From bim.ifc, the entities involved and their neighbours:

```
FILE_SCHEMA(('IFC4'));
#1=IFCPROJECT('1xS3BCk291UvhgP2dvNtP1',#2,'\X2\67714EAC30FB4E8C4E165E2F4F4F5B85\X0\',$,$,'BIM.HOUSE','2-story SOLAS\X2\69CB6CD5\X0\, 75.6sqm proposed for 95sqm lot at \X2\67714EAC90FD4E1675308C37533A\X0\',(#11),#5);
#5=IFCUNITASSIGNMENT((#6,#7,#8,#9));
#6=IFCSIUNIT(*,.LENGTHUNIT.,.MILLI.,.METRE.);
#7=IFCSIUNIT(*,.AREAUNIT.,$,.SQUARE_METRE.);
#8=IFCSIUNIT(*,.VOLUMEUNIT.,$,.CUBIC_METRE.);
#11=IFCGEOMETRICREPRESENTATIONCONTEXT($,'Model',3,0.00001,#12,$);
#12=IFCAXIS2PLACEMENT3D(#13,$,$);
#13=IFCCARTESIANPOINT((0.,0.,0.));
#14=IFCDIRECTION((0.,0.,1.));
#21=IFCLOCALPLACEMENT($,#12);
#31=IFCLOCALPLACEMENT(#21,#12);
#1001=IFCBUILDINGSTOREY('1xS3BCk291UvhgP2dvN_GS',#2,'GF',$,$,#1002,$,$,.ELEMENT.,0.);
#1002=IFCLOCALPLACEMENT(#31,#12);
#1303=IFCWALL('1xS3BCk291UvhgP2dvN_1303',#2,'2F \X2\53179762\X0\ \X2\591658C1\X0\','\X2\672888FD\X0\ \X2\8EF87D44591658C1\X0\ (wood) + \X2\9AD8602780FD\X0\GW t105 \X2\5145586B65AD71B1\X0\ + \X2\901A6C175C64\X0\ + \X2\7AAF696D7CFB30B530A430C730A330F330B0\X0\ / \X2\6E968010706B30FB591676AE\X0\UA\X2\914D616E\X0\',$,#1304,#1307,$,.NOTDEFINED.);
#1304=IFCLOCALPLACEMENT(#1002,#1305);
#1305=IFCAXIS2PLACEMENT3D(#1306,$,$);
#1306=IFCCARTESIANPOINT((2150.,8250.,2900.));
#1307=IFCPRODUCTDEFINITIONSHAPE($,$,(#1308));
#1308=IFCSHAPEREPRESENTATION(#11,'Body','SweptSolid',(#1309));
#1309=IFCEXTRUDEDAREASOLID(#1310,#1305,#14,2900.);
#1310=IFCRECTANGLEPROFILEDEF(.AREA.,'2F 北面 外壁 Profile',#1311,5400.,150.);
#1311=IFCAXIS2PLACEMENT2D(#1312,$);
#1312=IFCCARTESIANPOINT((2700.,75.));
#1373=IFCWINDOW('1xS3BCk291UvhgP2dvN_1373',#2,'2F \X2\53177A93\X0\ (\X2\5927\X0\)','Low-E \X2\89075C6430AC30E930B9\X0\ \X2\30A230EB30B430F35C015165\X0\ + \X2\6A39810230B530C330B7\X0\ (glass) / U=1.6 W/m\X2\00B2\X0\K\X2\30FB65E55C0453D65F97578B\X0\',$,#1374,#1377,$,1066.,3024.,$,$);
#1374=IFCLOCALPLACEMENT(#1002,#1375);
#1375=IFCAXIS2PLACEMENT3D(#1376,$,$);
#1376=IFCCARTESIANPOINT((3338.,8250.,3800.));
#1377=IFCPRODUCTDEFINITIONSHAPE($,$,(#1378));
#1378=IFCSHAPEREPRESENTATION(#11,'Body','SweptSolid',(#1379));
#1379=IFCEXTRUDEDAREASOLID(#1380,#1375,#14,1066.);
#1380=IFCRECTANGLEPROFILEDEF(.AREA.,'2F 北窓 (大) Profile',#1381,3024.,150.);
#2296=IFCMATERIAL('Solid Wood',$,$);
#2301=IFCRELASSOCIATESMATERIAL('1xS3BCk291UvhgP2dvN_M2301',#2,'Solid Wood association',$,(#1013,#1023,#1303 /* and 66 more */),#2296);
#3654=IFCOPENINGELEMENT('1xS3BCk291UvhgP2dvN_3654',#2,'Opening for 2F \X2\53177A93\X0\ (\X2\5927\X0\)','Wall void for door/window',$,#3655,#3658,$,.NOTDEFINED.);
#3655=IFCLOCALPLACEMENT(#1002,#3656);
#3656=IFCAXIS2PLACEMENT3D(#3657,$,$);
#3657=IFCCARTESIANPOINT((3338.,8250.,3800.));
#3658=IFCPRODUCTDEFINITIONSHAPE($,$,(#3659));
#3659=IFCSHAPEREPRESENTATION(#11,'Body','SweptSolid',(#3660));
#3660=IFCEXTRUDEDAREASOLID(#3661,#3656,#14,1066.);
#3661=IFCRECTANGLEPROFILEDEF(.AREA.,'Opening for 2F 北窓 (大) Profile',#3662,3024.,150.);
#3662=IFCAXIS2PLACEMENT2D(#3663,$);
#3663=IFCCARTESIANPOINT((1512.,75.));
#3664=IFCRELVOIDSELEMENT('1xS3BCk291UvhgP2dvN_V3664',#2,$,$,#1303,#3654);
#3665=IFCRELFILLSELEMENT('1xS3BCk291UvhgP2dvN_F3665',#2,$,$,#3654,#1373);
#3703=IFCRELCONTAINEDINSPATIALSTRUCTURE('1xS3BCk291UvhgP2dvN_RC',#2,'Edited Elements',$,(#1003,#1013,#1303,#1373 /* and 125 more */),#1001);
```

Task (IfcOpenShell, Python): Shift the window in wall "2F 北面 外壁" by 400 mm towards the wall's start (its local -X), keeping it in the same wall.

```python
import ifcopenshell
import ifcopenshell.api.geometry
import ifcopenshell.util.placement
import ifcopenshell.util.unit

model = ifcopenshell.open("bim.ifc")
unit_scale = ifcopenshell.util.unit.calculate_unit_scale(model)

window = model.by_guid("1xS3BCk291UvhgP2dvN_1373")
opening = window.FillsVoids[0].RelatingOpeningElement
wall = opening.VoidsElements[0].RelatingBuildingElement

wall_matrix = ifcopenshell.util.placement.get_local_placement(wall.ObjectPlacement)
shift = wall_matrix[:3, 0] * -0.4 / unit_scale
before = ifcopenshell.util.placement.get_local_placement(window.ObjectPlacement)[:3, 3].copy()

# The window is not placed relative to its opening, so move both.
for product in (opening, window):
    matrix = ifcopenshell.util.placement.get_local_placement(product.ObjectPlacement)
    matrix[:3, 3] += shift
    ifcopenshell.api.geometry.edit_object_placement(model, product=product, matrix=matrix, is_si=False)

after = ifcopenshell.util.placement.get_local_placement(window.ObjectPlacement)[:3, 3]
print("window moved by", (after - before).round(3) + 0.0)

model.write("bim_edited.ifc")
```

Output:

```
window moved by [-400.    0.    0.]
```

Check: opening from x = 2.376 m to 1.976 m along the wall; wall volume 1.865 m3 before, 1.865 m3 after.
